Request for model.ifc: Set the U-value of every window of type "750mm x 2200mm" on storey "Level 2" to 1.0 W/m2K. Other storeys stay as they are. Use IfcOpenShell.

First a look at what the model holds.

```python
import ifcopenshell
import ifcopenshell.util.element

model = ifcopenshell.open("model.ifc")
print(model.schema)
storey = next(s for s in model.by_type("IfcBuildingStorey") if s.Name == "Level 2")
windows = [e for e in ifcopenshell.util.element.get_decomposition(storey) if e.is_a("IfcWindow")]
seen = {}
for e in windows:
    element_type = ifcopenshell.util.element.get_type(e)
    key = (element_type.Name if element_type != e and element_type else None, ifcopenshell.util.element.get_pset(e, "Pset_WindowCommon", "ThermalTransmittance"))
    seen[key] = seen.get(key, 0) + 1
for (name, value), count in sorted(seen.items(), key=str):
    print(count, "x", name, "|", value)
```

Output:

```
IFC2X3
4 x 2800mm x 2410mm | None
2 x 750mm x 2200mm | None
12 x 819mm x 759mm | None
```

```python
import ifcopenshell
import ifcopenshell.api.pset
import ifcopenshell.util.element

model = ifcopenshell.open("model.ifc")

storey = next(s for s in model.by_type("IfcBuildingStorey") if s.Name == "Level 2")
windows = [e for e in ifcopenshell.util.element.get_decomposition(storey) if e.is_a("IfcWindow")]

count = 0
for e in windows:
    element_type = ifcopenshell.util.element.get_type(e)
    if element_type in (None, e) or element_type.Name != "750mm x 2200mm":
        continue
    # add_pset returns the element's existing set when there is one.
    pset = ifcopenshell.api.pset.add_pset(model, product=e, name="Pset_WindowCommon")
    ifcopenshell.api.pset.edit_pset(model, pset=pset, properties={"ThermalTransmittance": 1.0})
    count += 1

print(count, "windows updated")

model.write("model_v2.ifc")
```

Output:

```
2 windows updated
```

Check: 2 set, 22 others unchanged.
